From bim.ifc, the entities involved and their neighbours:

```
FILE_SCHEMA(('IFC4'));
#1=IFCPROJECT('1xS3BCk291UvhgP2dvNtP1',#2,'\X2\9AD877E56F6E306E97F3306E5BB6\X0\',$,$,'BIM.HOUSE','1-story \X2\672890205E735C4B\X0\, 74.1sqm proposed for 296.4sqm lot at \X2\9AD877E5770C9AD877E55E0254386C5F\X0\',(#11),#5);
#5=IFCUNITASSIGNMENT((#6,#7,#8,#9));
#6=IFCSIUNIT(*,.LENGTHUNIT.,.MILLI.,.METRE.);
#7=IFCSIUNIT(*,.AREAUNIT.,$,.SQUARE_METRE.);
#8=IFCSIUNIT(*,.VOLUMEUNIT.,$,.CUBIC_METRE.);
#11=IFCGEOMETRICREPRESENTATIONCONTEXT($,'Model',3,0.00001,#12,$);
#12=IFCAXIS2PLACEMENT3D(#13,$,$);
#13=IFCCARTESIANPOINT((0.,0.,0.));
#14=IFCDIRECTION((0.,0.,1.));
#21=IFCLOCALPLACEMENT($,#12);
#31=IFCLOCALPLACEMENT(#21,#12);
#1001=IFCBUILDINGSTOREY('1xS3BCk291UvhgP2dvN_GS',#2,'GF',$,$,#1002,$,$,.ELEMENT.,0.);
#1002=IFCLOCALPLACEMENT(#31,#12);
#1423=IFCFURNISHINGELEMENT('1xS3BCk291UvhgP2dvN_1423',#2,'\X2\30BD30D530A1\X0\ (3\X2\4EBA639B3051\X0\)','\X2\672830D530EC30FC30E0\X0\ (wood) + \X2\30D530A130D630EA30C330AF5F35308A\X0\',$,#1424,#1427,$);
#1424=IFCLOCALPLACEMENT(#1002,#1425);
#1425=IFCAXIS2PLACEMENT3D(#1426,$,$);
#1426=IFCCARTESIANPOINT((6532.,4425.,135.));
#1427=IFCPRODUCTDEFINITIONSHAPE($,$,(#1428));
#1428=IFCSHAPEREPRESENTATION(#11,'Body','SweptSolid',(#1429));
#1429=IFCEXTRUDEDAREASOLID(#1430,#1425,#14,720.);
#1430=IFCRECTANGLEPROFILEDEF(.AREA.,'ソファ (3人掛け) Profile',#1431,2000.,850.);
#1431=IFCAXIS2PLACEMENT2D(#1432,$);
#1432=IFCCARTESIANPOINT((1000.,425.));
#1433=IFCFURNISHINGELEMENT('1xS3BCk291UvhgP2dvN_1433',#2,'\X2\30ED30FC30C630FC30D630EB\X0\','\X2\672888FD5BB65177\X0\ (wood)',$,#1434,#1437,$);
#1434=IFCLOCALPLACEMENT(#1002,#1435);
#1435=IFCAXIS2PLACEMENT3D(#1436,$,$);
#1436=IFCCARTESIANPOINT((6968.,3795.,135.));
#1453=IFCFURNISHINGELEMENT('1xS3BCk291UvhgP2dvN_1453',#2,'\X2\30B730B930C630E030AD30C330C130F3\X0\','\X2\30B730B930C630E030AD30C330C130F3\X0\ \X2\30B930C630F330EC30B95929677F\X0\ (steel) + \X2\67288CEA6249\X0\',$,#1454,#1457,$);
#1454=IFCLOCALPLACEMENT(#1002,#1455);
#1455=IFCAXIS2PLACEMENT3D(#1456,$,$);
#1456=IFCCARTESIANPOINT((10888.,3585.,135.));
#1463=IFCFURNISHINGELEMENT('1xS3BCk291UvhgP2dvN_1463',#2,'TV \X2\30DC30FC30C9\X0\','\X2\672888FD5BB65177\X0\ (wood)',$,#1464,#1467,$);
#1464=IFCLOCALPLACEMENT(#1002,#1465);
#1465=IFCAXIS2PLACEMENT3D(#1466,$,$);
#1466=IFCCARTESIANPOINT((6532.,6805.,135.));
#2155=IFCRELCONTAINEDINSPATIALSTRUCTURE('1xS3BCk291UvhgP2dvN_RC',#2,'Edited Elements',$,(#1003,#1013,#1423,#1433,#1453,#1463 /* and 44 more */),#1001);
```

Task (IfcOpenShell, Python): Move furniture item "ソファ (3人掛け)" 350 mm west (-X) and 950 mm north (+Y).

```python
import ifcopenshell
import ifcopenshell.api.geometry
import ifcopenshell.util.placement
import ifcopenshell.util.unit

model = ifcopenshell.open("bim.ifc")
unit_scale = ifcopenshell.util.unit.calculate_unit_scale(model)

item = model.by_guid("1xS3BCk291UvhgP2dvN_1423")
matrix = ifcopenshell.util.placement.get_local_placement(item.ObjectPlacement)
matrix[0, 3] -= 0.35 / unit_scale
matrix[1, 3] += 0.95 / unit_scale
ifcopenshell.api.geometry.edit_object_placement(model, product=item, matrix=matrix, is_si=False)

print(ifcopenshell.util.placement.get_local_placement(item.ObjectPlacement).round(3) + 0.0)

model.write("bim_v2.ifc")
```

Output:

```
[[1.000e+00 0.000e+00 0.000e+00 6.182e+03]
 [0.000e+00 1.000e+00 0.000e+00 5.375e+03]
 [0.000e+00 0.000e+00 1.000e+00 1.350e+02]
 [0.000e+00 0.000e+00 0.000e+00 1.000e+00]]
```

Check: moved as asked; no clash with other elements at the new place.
